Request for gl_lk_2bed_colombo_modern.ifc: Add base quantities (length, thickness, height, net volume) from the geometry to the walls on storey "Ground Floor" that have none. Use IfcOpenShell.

First a look at what the model holds.

```python
import ifcopenshell
import ifcopenshell.util.element
import ifcopenshell.util.unit

model = ifcopenshell.open("gl_lk_2bed_colombo_modern.ifc")
print(model.schema)
for unit_type in ("LENGTHUNIT", "AREAUNIT", "VOLUMEUNIT"):
    print(unit_type, ifcopenshell.util.unit.calculate_unit_scale(model, unit_type))
storey = next(s for s in model.by_type("IfcBuildingStorey") if s.Name == "Ground Floor")
walls = [e for e in ifcopenshell.util.element.get_decomposition(storey) if e.is_a("IfcWall")]
for e in sorted(walls, key=lambda e: e.id()):
    print(e.id(), e.is_a(), e.Name, list(ifcopenshell.util.element.get_psets(e, qtos_only=True)), sep=" | ")
```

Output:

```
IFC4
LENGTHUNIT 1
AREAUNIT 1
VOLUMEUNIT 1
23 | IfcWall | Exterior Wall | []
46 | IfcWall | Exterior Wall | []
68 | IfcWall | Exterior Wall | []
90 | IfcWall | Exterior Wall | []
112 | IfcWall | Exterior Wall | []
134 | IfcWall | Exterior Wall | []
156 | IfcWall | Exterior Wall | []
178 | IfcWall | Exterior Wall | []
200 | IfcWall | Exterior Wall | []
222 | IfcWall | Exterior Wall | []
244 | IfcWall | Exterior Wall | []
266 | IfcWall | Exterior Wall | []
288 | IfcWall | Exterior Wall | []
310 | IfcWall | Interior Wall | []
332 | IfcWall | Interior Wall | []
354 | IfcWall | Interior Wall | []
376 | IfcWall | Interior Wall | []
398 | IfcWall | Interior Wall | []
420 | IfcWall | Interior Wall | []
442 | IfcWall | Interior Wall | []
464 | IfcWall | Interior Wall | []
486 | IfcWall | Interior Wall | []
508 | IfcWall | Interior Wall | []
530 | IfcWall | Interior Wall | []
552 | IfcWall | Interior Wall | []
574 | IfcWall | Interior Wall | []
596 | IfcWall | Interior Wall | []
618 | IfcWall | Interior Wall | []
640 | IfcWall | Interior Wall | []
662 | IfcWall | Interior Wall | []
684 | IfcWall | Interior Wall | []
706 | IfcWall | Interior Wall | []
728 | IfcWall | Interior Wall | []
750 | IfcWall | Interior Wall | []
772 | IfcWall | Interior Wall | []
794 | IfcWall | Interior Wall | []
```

```python
import ifcopenshell
import ifcopenshell.api.pset
import ifcopenshell.geom
import ifcopenshell.util.element
import ifcopenshell.util.shape
import ifcopenshell.util.unit

model = ifcopenshell.open("gl_lk_2bed_colombo_modern.ifc")
unit_scale = ifcopenshell.util.unit.calculate_unit_scale(model)
volume_scale = ifcopenshell.util.unit.calculate_unit_scale(model, "VOLUMEUNIT")
settings = ifcopenshell.geom.settings()

storey = next(s for s in model.by_type("IfcBuildingStorey") if s.Name == "Ground Floor")
walls = [e for e in ifcopenshell.util.element.get_decomposition(storey) if e.is_a("IfcWall")]

for e in sorted(walls, key=lambda e: e.id()):
    if ifcopenshell.util.element.get_psets(e, qtos_only=True, should_inherit=False):
        continue
    # Geometry comes back in metres, in the element's own axes.
    shape = ifcopenshell.geom.create_shape(settings, e)
    values = {
        "Length": ifcopenshell.util.shape.get_x(shape.geometry) / unit_scale,
        "Width": ifcopenshell.util.shape.get_y(shape.geometry) / unit_scale,
        "Height": ifcopenshell.util.shape.get_z(shape.geometry) / unit_scale,
        "NetVolume": ifcopenshell.util.shape.get_volume(shape.geometry) / volume_scale,
    }
    qto = ifcopenshell.api.pset.add_qto(model, product=e, name="Qto_WallBaseQuantities")
    ifcopenshell.api.pset.edit_qto(model, qto=qto, properties=values)
    print(e.id(), {k: round(v, 3) for k, v in values.items()})

model.write("gl_lk_2bed_colombo_modern_v2.ifc")
```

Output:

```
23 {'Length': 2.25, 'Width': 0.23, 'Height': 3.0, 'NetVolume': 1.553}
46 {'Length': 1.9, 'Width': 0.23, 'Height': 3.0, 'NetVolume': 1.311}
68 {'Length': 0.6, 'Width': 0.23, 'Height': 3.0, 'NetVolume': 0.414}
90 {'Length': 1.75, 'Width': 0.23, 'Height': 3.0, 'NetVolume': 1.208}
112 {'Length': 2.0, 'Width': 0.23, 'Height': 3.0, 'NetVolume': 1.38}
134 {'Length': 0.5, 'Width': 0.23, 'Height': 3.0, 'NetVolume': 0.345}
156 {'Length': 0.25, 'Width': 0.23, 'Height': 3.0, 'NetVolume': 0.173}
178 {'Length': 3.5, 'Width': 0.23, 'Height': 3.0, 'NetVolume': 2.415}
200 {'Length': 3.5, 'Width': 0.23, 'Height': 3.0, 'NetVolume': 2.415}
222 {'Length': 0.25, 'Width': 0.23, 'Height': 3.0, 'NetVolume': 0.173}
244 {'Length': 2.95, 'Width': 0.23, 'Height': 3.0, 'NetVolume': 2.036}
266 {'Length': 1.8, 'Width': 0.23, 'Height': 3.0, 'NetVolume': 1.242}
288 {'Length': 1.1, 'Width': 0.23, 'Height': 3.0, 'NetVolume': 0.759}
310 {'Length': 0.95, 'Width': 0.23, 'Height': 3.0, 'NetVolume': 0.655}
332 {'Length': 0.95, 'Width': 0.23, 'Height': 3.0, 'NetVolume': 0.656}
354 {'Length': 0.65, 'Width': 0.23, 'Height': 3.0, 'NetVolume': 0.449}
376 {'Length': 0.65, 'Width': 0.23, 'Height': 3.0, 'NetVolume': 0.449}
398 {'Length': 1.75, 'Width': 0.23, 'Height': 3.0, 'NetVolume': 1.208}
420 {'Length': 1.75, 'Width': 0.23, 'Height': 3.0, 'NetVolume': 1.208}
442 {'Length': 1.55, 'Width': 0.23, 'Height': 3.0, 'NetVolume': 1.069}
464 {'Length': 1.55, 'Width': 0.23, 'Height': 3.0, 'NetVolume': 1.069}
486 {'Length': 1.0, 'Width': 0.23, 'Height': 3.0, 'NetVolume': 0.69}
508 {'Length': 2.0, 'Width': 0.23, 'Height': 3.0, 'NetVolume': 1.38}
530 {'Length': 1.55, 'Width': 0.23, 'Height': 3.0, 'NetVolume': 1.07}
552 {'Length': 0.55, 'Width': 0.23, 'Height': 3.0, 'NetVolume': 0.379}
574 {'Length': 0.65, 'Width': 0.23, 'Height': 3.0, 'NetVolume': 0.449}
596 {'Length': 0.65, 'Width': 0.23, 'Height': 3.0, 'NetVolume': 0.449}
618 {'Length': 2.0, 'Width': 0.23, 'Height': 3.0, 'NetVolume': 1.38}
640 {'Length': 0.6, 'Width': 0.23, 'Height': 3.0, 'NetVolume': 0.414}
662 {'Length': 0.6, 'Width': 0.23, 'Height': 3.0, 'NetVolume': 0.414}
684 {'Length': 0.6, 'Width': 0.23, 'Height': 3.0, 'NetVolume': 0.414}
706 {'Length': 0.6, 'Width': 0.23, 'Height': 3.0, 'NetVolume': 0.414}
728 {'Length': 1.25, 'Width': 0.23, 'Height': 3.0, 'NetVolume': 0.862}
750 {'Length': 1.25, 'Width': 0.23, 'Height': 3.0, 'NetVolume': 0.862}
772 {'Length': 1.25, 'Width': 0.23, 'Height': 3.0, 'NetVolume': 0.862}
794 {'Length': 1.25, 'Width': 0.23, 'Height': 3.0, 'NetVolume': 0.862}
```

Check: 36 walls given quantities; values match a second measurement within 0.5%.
